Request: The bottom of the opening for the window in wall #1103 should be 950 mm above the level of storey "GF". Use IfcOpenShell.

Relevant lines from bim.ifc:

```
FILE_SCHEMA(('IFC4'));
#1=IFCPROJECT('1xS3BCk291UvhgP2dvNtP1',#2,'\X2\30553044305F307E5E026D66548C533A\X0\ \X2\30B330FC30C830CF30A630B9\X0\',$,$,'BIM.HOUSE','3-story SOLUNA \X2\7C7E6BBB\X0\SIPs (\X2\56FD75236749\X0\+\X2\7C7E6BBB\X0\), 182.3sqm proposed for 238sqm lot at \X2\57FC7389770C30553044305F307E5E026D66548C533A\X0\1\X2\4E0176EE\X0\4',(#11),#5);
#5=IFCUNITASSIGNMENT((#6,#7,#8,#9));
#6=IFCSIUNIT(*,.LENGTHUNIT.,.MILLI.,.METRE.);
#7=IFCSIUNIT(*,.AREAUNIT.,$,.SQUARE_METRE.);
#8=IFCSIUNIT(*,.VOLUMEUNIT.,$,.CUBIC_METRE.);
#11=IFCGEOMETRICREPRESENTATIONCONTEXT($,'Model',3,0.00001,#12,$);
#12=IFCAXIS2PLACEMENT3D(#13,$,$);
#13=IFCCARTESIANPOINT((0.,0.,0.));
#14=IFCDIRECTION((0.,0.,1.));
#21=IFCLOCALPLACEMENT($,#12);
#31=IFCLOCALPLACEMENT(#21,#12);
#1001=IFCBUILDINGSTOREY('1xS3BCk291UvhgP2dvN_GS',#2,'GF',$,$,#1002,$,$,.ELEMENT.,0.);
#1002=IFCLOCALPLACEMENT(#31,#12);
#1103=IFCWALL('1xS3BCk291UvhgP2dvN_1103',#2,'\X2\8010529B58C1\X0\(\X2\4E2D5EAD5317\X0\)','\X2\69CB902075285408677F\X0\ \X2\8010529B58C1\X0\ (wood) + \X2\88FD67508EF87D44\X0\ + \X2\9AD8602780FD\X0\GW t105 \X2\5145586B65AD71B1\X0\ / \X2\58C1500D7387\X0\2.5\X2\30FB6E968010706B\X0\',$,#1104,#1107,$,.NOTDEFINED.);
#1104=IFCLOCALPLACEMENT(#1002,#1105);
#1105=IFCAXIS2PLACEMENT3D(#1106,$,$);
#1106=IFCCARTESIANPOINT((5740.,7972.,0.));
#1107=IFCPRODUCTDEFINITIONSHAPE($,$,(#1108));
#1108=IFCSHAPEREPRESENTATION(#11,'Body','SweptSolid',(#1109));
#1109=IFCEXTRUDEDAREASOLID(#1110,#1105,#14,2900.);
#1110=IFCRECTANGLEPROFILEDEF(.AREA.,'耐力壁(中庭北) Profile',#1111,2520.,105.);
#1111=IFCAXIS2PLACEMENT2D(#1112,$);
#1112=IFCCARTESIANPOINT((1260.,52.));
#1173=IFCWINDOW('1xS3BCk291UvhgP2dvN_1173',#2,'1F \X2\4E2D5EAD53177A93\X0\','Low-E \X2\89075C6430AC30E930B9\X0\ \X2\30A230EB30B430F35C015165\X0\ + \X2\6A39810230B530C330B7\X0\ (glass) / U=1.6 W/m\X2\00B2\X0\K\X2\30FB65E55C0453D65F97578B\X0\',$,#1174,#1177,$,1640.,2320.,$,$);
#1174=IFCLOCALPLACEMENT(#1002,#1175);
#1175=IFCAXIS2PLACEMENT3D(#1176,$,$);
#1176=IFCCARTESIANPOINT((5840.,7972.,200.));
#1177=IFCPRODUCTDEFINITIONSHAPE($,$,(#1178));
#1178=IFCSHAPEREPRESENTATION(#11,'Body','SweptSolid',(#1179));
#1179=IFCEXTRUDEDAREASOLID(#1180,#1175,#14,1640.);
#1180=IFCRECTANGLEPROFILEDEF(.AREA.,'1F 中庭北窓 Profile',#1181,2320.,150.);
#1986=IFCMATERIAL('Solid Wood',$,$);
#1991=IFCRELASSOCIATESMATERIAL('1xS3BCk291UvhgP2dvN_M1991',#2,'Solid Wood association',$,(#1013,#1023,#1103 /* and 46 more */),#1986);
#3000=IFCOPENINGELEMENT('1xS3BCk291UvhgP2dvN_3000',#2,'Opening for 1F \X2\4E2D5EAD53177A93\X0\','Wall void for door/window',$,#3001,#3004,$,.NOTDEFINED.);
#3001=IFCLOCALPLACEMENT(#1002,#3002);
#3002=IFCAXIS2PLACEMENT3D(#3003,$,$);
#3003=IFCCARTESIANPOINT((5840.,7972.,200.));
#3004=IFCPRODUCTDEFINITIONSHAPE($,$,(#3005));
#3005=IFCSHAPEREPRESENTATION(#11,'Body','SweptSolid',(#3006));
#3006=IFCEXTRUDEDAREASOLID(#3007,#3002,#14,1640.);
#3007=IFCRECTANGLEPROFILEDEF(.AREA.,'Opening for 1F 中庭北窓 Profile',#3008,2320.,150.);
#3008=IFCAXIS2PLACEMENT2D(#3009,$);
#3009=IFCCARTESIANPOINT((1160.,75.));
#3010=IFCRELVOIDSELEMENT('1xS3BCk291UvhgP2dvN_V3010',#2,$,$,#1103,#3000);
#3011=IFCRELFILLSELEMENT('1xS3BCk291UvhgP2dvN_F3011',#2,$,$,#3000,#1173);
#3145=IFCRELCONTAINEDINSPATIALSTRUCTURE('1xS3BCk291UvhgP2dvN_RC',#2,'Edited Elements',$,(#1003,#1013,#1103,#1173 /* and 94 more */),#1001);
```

```python
import numpy as np
import ifcopenshell
import ifcopenshell.api.geometry
import ifcopenshell.geom
import ifcopenshell.util.element
import ifcopenshell.util.placement
import ifcopenshell.util.shape
import ifcopenshell.util.unit

model = ifcopenshell.open("bim.ifc")
unit_scale = ifcopenshell.util.unit.calculate_unit_scale(model)

window = model.by_guid("1xS3BCk291UvhgP2dvN_1173")
opening = window.FillsVoids[0].RelatingOpeningElement
storey = ifcopenshell.util.element.get_container(window, ifc_class="IfcBuildingStorey")
level = ifcopenshell.util.placement.get_local_placement(storey.ObjectPlacement)[2, 3]

# The opening's origin need not be at the sill, so measure its lowest point.
shape = ifcopenshell.geom.create_shape(ifcopenshell.geom.settings(), opening)
bottom = ifcopenshell.util.shape.get_shape_bottom_elevation(shape, shape.geometry) / unit_scale
dz = level + 0.95 / unit_scale - bottom

shift = np.array([0.0, 0.0, dz])
# The window is not placed relative to its opening, so move both.
for product in (opening, window):
    matrix = ifcopenshell.util.placement.get_local_placement(product.ObjectPlacement)
    matrix[:3, 3] += shift
    ifcopenshell.api.geometry.edit_object_placement(model, product=product, matrix=matrix, is_si=False)

print(f"moved by {dz * unit_scale:+.3f} m")

model.write("bim_v2.ifc")
```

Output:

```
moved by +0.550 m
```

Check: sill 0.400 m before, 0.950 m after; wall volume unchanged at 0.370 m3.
